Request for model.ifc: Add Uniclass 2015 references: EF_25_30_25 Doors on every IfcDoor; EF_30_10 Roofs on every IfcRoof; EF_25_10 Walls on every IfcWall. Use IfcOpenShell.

First a look at what the model holds.

```python
import ifcopenshell

model = ifcopenshell.open("model.ifc")
print(model.schema)
print("classifications:", [c.Name for c in model.by_type("IfcClassification")])
for ifc_class in ("IfcDoor", "IfcRoof", "IfcStair", "IfcWall", "IfcWindow"):
    print(ifc_class, len(model.by_type(ifc_class)))
```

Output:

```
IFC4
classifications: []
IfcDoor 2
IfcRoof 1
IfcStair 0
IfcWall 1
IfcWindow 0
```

```python
import ifcopenshell
import ifcopenshell.api.classification

model = ifcopenshell.open("model.ifc")

system = ifcopenshell.api.classification.add_classification(model, classification="Uniclass 2015")

codes = {
    "IfcDoor": ("EF_25_30_25", "Doors"),
    "IfcRoof": ("EF_30_10", "Roofs"),
    "IfcWall": ("EF_25_10", "Walls"),
}
for ifc_class, (code, name) in codes.items():
    products = model.by_type(ifc_class)
    ifcopenshell.api.classification.add_reference(
        model, products=products, classification=system, identification=code, name=name
    )
    print(code, len(products))

model.write("model_v2.ifc")
```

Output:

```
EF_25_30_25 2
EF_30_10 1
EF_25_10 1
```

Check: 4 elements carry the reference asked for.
